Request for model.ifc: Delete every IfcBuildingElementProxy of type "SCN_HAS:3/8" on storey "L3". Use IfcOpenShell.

First a look at what the model holds.

```python
import ifcopenshell
import ifcopenshell.util.element

model = ifcopenshell.open("model.ifc")
print(model.schema)
storey = next(s for s in model.by_type("IfcBuildingStorey") if s.Name == "L3")
proxies = [e for e in ifcopenshell.util.element.get_decomposition(storey) if e.is_a("IfcBuildingElementProxy")]
seen = {}
for e in proxies:
    element_type = ifcopenshell.util.element.get_type(e)
    name = element_type.Name if element_type not in (None, e) else None
    seen[name] = seen.get(name, 0) + 1
for name, count in sorted(seen.items(), key=str):
    print(count, "x", name)
```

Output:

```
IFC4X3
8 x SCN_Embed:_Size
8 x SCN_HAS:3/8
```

```python
import ifcopenshell
import ifcopenshell.api.root
import ifcopenshell.util.element

model = ifcopenshell.open("model.ifc")

storey = next(s for s in model.by_type("IfcBuildingStorey") if s.Name == "L3")
proxies = [e for e in ifcopenshell.util.element.get_decomposition(storey) if e.is_a("IfcBuildingElementProxy")]
targets = [e for e in proxies if (t := ifcopenshell.util.element.get_type(e)) not in (None, e) and t.Name == "SCN_HAS:3/8"]

for e in targets:
    ifcopenshell.api.root.remove_product(model, product=e)
print(len(targets), "removed")

model.write("model-out.ifc")
```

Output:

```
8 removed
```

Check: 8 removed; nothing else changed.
